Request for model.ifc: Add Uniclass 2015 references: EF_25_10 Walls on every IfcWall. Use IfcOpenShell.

First a look at what the model holds.

```python
import ifcopenshell

model = ifcopenshell.open("model.ifc")
print(model.schema)
print("classifications:", [c.Name for c in model.by_type("IfcClassification")])
for ifc_class in ("IfcDoor", "IfcRoof", "IfcStair", "IfcWall", "IfcWindow"):
    print(ifc_class, len(model.by_type(ifc_class)))
```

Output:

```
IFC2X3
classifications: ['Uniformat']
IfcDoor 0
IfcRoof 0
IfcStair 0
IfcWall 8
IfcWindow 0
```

```python
import ifcopenshell
import ifcopenshell.api.classification

model = ifcopenshell.open("model.ifc")

# IFC2X3 requires Source and Edition and has no link from the project to the system.
system = model.create_entity("IfcClassification", Source="NBS", Edition="2015", Name="Uniclass 2015")

codes = {
    "IfcWall": ("EF_25_10", "Walls"),
}
for ifc_class, (code, name) in codes.items():
    products = model.by_type(ifc_class)
    ifcopenshell.api.classification.add_reference(
        model, products=products, classification=system, identification=code, name=name
    )
    print(code, len(products))

model.write("model_edited.ifc")
```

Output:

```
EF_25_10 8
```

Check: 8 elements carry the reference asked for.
